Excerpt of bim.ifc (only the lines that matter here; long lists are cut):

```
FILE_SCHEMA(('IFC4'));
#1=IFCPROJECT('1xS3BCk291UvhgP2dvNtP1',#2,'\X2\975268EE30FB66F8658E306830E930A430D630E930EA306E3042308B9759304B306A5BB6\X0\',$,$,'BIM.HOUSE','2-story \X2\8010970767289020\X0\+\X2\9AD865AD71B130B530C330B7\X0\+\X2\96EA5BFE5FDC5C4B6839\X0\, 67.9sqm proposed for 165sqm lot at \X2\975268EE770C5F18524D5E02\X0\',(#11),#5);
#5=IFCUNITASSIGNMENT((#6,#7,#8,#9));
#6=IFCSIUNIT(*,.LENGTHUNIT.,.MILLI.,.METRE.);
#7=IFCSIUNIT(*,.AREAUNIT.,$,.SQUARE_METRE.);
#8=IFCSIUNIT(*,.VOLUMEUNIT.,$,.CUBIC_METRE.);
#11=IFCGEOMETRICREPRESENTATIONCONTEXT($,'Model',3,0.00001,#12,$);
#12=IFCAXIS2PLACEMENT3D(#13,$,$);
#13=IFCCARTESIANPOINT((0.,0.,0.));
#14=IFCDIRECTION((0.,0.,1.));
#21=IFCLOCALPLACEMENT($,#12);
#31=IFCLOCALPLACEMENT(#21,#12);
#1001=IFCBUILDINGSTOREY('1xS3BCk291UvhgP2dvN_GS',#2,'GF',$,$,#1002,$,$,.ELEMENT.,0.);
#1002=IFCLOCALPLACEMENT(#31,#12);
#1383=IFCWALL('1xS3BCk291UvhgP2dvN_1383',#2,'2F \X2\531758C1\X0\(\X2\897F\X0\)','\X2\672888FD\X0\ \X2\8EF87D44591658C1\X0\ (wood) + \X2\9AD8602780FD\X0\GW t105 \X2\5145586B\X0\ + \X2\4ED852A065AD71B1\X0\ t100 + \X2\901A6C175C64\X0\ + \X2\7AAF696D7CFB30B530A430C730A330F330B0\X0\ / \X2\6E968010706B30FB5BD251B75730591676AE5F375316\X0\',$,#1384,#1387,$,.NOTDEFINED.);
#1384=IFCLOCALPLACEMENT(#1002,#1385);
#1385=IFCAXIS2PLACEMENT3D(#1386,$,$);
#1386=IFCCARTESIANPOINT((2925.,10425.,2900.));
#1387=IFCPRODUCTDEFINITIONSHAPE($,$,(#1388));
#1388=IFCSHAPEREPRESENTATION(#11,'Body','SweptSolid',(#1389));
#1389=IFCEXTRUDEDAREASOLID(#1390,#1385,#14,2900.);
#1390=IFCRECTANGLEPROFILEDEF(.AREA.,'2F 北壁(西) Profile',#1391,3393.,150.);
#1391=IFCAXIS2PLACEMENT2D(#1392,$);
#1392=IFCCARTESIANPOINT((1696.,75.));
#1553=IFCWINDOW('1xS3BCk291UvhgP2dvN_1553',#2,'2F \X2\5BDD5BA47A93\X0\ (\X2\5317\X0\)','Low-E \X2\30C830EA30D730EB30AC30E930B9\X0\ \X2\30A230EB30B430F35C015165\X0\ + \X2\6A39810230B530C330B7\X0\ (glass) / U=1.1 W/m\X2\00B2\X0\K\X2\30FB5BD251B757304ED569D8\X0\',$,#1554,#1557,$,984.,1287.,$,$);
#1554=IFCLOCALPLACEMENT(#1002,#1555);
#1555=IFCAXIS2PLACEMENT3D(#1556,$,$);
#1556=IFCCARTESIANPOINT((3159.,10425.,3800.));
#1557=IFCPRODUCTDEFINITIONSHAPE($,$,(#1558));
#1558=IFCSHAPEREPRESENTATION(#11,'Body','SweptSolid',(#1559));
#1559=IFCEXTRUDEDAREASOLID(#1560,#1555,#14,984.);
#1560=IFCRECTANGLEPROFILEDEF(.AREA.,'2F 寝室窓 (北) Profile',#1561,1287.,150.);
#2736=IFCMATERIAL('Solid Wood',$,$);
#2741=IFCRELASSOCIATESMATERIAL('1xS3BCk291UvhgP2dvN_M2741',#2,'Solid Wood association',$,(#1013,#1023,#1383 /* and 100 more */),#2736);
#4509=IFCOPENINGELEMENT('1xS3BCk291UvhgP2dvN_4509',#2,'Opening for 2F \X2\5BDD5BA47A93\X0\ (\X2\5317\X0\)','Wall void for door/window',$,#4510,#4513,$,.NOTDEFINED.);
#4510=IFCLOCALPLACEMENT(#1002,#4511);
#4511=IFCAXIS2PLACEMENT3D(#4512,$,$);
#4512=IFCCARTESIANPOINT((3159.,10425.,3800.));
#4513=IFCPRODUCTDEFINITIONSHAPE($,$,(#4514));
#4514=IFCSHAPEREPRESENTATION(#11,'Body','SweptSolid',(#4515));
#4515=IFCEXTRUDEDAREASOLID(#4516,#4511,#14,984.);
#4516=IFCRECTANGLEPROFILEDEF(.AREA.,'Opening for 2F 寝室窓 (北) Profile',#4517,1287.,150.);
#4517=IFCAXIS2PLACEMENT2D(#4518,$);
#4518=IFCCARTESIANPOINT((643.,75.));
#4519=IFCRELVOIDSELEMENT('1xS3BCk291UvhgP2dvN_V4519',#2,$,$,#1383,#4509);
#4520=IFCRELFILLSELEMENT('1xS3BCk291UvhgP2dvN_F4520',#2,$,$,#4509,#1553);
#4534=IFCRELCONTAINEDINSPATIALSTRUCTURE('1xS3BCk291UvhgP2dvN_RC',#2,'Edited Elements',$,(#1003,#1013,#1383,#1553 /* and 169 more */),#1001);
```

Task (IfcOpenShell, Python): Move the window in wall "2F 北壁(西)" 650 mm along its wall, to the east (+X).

```python
import ifcopenshell
import ifcopenshell.api.geometry
import ifcopenshell.util.placement

model = ifcopenshell.open("bim.ifc")

window = model.by_id(1553)
opening = window.FillsVoids[0].RelatingOpeningElement
wall = opening.VoidsElements[0].RelatingBuildingElement

wall_matrix = ifcopenshell.util.placement.get_local_placement(wall.ObjectPlacement)
shift = wall_matrix[:3, 0] * 650.0
before = ifcopenshell.util.placement.get_local_placement(window.ObjectPlacement)[:3, 3].copy()

# The window is not placed relative to its opening, so move both.
for product in (opening, window):
    matrix = ifcopenshell.util.placement.get_local_placement(product.ObjectPlacement)
    matrix[:3, 3] += shift
    ifcopenshell.api.geometry.edit_object_placement(model, product=product, matrix=matrix, is_si=False)

after = ifcopenshell.util.placement.get_local_placement(window.ObjectPlacement)[:3, 3]
print("window moved by", (after - before).round(3) + 0.0)

model.write("bim_rev.ifc")
```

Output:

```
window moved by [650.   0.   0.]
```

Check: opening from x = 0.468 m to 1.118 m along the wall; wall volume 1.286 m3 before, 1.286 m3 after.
